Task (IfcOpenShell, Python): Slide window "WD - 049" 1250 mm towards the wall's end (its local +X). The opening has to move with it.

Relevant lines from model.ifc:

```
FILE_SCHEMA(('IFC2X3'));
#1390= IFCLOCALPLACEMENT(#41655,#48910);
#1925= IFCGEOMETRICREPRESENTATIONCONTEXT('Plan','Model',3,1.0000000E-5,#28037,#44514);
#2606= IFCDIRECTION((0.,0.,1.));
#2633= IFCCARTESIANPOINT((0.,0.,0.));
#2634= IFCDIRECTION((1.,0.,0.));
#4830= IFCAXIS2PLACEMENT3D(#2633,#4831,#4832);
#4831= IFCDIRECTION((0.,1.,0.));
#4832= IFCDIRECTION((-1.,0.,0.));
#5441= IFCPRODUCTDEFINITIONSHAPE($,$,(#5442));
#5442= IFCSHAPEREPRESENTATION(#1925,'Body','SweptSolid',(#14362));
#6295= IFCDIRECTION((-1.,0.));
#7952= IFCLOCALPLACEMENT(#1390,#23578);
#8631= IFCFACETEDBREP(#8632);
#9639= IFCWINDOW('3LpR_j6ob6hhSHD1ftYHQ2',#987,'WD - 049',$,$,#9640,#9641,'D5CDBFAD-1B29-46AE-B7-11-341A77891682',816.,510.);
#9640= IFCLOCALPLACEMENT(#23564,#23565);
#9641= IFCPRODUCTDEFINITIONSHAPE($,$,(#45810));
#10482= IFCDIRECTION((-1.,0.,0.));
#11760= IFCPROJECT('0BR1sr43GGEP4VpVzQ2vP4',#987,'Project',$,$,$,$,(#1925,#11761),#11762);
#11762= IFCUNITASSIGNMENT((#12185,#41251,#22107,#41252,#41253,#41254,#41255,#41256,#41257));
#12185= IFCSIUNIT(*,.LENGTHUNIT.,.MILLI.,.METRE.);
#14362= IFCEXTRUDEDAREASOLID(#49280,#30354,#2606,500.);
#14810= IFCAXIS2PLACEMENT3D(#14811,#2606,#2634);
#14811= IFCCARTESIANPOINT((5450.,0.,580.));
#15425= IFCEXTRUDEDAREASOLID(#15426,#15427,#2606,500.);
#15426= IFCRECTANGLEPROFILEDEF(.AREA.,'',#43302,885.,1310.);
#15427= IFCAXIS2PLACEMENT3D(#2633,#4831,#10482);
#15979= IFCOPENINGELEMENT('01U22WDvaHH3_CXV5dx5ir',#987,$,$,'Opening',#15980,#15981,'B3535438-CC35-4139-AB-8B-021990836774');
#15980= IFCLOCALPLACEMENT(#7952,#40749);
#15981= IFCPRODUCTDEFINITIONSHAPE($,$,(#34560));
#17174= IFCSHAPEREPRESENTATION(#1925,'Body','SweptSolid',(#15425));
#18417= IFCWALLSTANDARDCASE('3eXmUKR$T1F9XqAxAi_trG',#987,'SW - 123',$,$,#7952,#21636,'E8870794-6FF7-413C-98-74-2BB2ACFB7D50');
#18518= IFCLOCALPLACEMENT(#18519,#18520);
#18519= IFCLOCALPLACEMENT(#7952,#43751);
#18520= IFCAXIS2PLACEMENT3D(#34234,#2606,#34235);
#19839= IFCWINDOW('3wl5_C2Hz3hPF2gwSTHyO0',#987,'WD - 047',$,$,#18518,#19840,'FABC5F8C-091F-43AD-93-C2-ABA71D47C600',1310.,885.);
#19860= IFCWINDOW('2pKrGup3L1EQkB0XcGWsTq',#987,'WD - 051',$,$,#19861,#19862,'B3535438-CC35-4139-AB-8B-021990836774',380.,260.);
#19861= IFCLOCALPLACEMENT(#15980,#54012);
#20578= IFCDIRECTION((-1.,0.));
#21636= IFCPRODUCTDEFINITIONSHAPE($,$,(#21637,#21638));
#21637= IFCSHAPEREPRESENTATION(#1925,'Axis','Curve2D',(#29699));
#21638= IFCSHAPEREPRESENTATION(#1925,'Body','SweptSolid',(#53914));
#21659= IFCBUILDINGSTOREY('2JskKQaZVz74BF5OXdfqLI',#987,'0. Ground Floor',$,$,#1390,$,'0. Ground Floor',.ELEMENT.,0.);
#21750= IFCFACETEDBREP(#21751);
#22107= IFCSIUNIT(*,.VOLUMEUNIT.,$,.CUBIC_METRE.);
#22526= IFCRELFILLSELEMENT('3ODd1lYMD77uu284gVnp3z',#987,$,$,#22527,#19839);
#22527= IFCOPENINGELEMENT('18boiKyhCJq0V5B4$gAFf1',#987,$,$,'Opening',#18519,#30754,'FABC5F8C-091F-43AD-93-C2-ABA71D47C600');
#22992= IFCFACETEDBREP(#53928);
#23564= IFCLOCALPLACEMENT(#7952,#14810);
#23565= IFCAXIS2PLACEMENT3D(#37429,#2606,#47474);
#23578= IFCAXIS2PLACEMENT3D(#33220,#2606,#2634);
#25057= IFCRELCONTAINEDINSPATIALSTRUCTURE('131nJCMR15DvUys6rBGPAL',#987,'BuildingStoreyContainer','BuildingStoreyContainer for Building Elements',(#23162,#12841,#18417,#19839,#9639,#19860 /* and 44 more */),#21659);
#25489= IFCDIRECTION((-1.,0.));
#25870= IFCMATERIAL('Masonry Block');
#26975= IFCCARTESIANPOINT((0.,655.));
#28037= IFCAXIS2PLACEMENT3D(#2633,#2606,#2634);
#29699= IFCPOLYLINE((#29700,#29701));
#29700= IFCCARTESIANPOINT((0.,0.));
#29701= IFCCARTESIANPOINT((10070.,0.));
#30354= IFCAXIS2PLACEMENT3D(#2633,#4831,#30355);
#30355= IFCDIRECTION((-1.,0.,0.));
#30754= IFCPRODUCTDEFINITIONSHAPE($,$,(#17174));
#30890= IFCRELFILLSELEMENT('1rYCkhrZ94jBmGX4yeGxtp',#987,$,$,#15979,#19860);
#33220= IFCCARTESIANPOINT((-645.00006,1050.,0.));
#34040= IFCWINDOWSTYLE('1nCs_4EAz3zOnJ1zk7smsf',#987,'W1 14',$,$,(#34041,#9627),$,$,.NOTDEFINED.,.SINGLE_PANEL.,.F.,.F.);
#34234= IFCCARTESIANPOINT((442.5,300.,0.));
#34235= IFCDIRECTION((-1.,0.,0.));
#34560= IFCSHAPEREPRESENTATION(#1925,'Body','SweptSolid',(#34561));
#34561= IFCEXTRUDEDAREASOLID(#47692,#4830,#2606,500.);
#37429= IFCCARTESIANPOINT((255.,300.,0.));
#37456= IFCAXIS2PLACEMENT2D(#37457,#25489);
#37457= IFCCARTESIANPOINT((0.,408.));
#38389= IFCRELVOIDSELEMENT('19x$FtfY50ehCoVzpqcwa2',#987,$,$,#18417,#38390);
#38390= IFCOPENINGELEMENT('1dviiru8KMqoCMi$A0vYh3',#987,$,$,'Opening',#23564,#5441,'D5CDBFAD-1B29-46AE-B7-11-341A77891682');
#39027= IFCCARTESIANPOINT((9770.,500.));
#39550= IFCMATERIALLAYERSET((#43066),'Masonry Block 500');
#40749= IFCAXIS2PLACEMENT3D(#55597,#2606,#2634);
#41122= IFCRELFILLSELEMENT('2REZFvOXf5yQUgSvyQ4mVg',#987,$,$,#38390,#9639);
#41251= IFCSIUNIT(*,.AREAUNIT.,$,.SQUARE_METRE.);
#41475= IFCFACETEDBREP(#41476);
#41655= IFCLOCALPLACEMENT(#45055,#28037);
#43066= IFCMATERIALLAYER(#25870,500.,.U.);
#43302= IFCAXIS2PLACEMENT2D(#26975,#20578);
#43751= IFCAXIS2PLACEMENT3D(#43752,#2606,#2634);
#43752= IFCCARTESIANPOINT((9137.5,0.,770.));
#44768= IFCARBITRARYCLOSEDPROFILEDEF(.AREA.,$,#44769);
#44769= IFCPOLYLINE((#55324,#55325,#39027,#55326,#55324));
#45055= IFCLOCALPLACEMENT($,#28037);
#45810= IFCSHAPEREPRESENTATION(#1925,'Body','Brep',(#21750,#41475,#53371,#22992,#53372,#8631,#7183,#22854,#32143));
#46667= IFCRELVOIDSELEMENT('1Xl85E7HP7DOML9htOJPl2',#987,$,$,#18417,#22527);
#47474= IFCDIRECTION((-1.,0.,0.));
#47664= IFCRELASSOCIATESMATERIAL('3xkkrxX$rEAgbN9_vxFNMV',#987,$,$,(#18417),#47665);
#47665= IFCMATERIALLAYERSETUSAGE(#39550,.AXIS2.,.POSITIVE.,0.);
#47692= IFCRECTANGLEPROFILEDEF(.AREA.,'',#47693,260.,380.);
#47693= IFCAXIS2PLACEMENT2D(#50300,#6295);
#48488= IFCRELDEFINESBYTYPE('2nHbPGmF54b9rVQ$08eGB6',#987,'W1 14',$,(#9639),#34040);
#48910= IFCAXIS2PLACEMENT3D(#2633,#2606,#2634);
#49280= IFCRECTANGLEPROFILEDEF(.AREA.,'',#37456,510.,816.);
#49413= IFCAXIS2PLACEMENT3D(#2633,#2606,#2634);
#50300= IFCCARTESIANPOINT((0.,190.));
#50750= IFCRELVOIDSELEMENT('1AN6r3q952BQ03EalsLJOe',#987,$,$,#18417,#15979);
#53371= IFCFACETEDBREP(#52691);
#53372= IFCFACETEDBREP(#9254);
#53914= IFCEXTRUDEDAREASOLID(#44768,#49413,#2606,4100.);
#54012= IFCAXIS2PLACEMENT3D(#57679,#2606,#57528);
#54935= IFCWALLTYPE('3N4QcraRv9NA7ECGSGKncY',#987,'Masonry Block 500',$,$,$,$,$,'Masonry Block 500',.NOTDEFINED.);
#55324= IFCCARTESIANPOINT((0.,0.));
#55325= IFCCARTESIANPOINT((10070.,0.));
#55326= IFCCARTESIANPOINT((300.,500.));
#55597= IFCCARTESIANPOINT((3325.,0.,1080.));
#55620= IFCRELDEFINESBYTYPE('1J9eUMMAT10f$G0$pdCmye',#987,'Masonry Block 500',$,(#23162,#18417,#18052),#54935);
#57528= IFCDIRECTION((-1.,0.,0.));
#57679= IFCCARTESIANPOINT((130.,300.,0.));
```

```python
import ifcopenshell
import ifcopenshell.api.geometry
import ifcopenshell.util.placement

model = ifcopenshell.open("model.ifc")

window = model.by_guid("3LpR_j6ob6hhSHD1ftYHQ2")
opening = window.FillsVoids[0].RelatingOpeningElement
wall = opening.VoidsElements[0].RelatingBuildingElement

wall_matrix = ifcopenshell.util.placement.get_local_placement(wall.ObjectPlacement)
shift = wall_matrix[:3, 0] * 1250.0
before = ifcopenshell.util.placement.get_local_placement(window.ObjectPlacement)[:3, 3].copy()

# The window is placed relative to its opening, so it follows when the opening moves.
matrix = ifcopenshell.util.placement.get_local_placement(opening.ObjectPlacement)
matrix[:3, 3] += shift
ifcopenshell.api.geometry.edit_object_placement(
    model, product=opening, matrix=matrix, is_si=False, should_transform_children=True
)

after = ifcopenshell.util.placement.get_local_placement(window.ObjectPlacement)[:3, 3]
print("window moved by", (after - before).round(3) + 0.0)

model.write("model_v2.ifc")
```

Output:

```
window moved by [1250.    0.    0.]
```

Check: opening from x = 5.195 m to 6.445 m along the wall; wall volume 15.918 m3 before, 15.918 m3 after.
